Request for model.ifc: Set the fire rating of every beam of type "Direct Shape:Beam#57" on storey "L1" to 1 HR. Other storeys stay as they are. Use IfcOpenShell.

First a look at what the model holds.

```python
import ifcopenshell
import ifcopenshell.util.element

model = ifcopenshell.open("model.ifc")
print(model.schema)
storey = next(s for s in model.by_type("IfcBuildingStorey") if s.Name == "L1")
beams = [e for e in ifcopenshell.util.element.get_decomposition(storey) if e.is_a("IfcBeam")]
seen = {}
for e in beams:
    element_type = ifcopenshell.util.element.get_type(e)
    key = (element_type.Name if element_type != e and element_type else None, ifcopenshell.util.element.get_pset(e, "Pset_BeamCommon", "FireRating"))
    seen[key] = seen.get(key, 0) + 1
for (name, value), count in sorted(seen.items(), key=str):
    print(count, "x", name, "|", value)
```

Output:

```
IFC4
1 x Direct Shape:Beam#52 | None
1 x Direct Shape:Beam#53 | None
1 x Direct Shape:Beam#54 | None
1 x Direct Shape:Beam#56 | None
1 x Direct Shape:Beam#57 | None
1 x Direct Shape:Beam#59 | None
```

```python
import ifcopenshell
import ifcopenshell.api.pset
import ifcopenshell.util.element

model = ifcopenshell.open("model.ifc")

storey = next(s for s in model.by_type("IfcBuildingStorey") if s.Name == "L1")
beams = [e for e in ifcopenshell.util.element.get_decomposition(storey) if e.is_a("IfcBeam")]

count = 0
for e in beams:
    element_type = ifcopenshell.util.element.get_type(e)
    if element_type in (None, e) or element_type.Name != "Direct Shape:Beam#57":
        continue
    # add_pset returns the element's existing set when there is one.
    pset = ifcopenshell.api.pset.add_pset(model, product=e, name="Pset_BeamCommon")
    ifcopenshell.api.pset.edit_pset(model, pset=pset, properties={"FireRating": "1 HR"})
    count += 1

print(count, "beams updated")

model.write("model_updated.ifc")
```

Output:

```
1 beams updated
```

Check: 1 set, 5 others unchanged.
